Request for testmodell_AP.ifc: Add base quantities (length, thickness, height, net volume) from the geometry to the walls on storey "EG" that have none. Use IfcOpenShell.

First a look at what the model holds.

```python
import ifcopenshell
import ifcopenshell.util.element
import ifcopenshell.util.unit

model = ifcopenshell.open("testmodell_AP.ifc")
print(model.schema)
for unit_type in ("LENGTHUNIT", "AREAUNIT", "VOLUMEUNIT"):
    print(unit_type, ifcopenshell.util.unit.calculate_unit_scale(model, unit_type))
storey = next(s for s in model.by_type("IfcBuildingStorey") if s.Name == "EG")
walls = [e for e in ifcopenshell.util.element.get_decomposition(storey) if e.is_a("IfcWall")]
for e in sorted(walls, key=lambda e: e.id()):
    print(e.id(), e.is_a(), e.Name, list(ifcopenshell.util.element.get_psets(e, qtos_only=True)), sep=" | ")
```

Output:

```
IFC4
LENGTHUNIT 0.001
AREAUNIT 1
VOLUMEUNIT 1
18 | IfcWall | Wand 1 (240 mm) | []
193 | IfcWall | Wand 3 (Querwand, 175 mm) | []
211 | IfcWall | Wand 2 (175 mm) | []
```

```python
import ifcopenshell
import ifcopenshell.api.pset
import ifcopenshell.geom
import ifcopenshell.util.element
import ifcopenshell.util.shape
import ifcopenshell.util.unit

model = ifcopenshell.open("testmodell_AP.ifc")
unit_scale = ifcopenshell.util.unit.calculate_unit_scale(model)
volume_scale = ifcopenshell.util.unit.calculate_unit_scale(model, "VOLUMEUNIT")
settings = ifcopenshell.geom.settings()

storey = next(s for s in model.by_type("IfcBuildingStorey") if s.Name == "EG")
walls = [e for e in ifcopenshell.util.element.get_decomposition(storey) if e.is_a("IfcWall")]

for e in sorted(walls, key=lambda e: e.id()):
    if ifcopenshell.util.element.get_psets(e, qtos_only=True, should_inherit=False):
        continue
    # Geometry comes back in metres, in the element's own axes.
    shape = ifcopenshell.geom.create_shape(settings, e)
    values = {
        "Length": ifcopenshell.util.shape.get_x(shape.geometry) / unit_scale,
        "Width": ifcopenshell.util.shape.get_y(shape.geometry) / unit_scale,
        "Height": ifcopenshell.util.shape.get_z(shape.geometry) / unit_scale,
        "NetVolume": ifcopenshell.util.shape.get_volume(shape.geometry) / volume_scale,
    }
    qto = ifcopenshell.api.pset.add_qto(model, product=e, name="Qto_WallBaseQuantities")
    ifcopenshell.api.pset.edit_qto(model, qto=qto, properties=values)
    print(e.id(), {k: round(v, 3) for k, v in values.items()})

model.write("testmodell_AP_edited.ifc")
```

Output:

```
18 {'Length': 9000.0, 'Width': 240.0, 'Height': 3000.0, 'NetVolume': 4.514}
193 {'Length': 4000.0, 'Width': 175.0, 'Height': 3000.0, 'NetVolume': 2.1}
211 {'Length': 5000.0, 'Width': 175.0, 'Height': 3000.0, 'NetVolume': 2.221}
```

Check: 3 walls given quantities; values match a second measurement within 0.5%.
